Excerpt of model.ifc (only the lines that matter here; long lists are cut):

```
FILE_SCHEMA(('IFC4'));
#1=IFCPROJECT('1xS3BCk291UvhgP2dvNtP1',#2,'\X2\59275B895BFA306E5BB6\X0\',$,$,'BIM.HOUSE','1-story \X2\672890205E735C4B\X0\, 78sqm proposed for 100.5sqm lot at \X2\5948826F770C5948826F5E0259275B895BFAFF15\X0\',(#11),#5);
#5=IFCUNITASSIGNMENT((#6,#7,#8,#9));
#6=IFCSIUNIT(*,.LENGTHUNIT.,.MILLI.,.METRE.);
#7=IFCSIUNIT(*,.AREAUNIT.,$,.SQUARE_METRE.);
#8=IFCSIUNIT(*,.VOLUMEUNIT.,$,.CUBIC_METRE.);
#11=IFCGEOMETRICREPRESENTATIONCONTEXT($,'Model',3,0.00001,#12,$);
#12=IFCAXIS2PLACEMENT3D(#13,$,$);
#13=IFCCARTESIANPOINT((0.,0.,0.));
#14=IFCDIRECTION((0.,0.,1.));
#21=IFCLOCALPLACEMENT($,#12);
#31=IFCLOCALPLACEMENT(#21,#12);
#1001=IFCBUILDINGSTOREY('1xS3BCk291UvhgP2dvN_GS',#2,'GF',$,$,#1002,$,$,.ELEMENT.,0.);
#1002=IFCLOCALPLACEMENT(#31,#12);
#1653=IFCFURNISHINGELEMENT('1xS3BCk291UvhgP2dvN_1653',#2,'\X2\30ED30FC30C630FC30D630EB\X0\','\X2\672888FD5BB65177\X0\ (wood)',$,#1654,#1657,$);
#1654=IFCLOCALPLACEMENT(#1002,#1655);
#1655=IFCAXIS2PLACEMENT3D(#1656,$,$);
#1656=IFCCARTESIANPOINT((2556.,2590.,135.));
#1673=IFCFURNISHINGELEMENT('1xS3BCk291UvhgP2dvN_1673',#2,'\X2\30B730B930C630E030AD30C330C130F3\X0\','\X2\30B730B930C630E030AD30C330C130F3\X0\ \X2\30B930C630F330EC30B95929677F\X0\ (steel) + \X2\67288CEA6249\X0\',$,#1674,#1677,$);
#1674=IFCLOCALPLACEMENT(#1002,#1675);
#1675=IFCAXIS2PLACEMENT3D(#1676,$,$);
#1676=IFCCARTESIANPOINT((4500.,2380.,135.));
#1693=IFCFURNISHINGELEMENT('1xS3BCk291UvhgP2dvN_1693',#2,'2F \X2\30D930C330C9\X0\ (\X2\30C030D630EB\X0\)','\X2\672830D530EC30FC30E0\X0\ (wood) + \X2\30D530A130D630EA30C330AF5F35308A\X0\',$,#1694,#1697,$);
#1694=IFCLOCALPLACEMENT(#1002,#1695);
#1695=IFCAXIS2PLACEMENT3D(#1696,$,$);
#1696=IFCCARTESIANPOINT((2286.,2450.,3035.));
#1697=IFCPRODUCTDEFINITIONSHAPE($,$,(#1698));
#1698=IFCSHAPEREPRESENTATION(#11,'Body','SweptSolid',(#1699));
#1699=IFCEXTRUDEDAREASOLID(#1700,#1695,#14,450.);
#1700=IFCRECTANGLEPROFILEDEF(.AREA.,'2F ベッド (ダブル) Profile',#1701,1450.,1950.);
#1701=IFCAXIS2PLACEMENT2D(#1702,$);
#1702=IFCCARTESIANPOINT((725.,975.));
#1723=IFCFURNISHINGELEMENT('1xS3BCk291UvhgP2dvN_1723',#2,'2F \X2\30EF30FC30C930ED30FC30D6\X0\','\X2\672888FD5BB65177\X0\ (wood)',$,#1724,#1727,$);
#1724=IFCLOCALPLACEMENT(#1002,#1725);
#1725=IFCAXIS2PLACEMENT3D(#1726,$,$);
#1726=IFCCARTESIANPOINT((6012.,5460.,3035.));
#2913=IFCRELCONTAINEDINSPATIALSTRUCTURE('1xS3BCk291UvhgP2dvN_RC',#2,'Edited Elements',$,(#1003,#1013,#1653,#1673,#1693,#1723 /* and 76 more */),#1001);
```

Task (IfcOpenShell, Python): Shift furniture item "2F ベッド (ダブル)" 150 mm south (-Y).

```python
import ifcopenshell
import ifcopenshell.api.geometry
import ifcopenshell.util.placement

model = ifcopenshell.open("model.ifc")

item = model.by_guid("1xS3BCk291UvhgP2dvN_1693")
matrix = ifcopenshell.util.placement.get_local_placement(item.ObjectPlacement)
matrix[1, 3] -= 150.0
ifcopenshell.api.geometry.edit_object_placement(model, product=item, matrix=matrix, is_si=False)

print(ifcopenshell.util.placement.get_local_placement(item.ObjectPlacement).round(3) + 0.0)

model.write("model-out.ifc")
```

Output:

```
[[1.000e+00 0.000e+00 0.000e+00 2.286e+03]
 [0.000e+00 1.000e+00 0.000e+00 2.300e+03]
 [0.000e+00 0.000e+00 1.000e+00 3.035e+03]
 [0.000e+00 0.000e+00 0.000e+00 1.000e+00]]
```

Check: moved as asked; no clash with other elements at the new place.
